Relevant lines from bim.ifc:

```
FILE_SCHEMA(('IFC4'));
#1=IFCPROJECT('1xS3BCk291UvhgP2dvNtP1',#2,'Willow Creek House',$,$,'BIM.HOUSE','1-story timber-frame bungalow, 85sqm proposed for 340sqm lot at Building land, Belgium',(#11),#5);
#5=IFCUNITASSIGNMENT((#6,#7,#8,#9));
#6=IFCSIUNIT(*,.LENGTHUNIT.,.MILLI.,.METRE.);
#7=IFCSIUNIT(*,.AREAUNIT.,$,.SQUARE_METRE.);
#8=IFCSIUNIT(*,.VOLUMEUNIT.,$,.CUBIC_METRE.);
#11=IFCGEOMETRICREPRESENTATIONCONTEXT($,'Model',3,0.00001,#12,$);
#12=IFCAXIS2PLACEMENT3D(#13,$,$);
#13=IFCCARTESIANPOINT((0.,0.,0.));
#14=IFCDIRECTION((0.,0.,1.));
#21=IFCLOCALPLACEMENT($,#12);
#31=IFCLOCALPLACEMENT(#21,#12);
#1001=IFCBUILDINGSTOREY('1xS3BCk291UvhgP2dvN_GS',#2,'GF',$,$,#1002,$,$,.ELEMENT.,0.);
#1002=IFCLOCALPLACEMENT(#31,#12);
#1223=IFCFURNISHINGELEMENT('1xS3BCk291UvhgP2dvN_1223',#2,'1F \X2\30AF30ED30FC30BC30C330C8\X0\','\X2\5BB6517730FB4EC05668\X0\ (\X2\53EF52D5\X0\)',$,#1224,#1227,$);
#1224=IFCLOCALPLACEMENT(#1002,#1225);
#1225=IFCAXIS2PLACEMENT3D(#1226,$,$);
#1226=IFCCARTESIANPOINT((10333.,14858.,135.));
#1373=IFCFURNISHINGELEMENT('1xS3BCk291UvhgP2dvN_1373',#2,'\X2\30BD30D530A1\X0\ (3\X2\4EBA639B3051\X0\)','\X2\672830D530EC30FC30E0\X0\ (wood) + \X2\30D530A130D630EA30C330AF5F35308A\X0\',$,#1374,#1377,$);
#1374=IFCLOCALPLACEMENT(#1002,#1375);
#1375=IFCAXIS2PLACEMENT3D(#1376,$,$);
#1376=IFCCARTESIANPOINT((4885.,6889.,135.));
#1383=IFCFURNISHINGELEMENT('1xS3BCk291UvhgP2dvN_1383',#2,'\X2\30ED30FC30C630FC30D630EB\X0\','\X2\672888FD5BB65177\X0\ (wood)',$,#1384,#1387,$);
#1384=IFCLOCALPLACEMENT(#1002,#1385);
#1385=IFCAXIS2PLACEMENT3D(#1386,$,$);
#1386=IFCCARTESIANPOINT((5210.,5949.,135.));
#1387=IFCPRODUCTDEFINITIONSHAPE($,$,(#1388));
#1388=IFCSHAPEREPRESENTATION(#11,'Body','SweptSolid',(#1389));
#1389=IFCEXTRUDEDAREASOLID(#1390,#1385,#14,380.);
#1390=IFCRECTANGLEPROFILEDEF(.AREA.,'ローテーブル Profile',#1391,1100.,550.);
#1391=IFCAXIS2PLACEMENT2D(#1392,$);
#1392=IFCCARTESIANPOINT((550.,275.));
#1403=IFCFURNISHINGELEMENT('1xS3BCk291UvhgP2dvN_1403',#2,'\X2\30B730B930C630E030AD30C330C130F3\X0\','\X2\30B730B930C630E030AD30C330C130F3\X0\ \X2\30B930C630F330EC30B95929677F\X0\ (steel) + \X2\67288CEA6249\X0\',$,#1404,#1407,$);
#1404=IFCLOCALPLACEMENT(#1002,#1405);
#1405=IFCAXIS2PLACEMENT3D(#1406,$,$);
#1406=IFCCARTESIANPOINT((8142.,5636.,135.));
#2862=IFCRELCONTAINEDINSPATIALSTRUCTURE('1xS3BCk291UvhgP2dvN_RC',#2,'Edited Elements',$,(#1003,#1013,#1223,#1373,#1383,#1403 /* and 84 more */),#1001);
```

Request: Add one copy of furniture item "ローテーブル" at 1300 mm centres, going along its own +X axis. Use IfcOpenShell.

```python
import ifcopenshell
import ifcopenshell.api.geometry
import ifcopenshell.api.root
import ifcopenshell.util.element
import ifcopenshell.util.placement
import ifcopenshell.util.unit

model = ifcopenshell.open("bim.ifc")
unit_scale = ifcopenshell.util.unit.calculate_unit_scale(model)


def reuse_history(source, copy):
    """copy_class also copies each property set's owner history, people and application; keep the originals."""
    for rel in copy.IsDefinedBy:
        if rel.is_a("IfcRelDefinesByProperties") and (history := rel.RelatingPropertyDefinition.OwnerHistory):
            rel.RelatingPropertyDefinition.OwnerHistory = source.OwnerHistory
            ifcopenshell.util.element.remove_deep2(model, history)


source = model.by_guid("1xS3BCk291UvhgP2dvN_1383")
base = ifcopenshell.util.placement.get_local_placement(source.ObjectPlacement)
step = base[:3, 0] * 1.3 / unit_scale

for i in range(1, 2):
    copy = ifcopenshell.api.root.copy_class(model, product=source)
    copy.Representation = ifcopenshell.util.element.copy_deep(
        model, source.Representation, exclude=["IfcGeometricRepresentationContext", "IfcRepresentationMap"]
    )
    reuse_history(source, copy)
    matrix = base.copy()
    matrix[:3, 3] += i * step
    print("added at", matrix[:3, 3].round(3) + 0.0)
    ifcopenshell.api.geometry.edit_object_placement(model, product=copy, matrix=matrix, is_si=False)

model.write("bim_rev.ifc")
```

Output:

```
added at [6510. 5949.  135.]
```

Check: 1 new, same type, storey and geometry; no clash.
